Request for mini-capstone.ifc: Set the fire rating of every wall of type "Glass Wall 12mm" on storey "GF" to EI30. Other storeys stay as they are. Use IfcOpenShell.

First a look at what the model holds.

```python
import ifcopenshell
import ifcopenshell.util.element

model = ifcopenshell.open("mini-capstone.ifc")
print(model.schema)
storey = next(s for s in model.by_type("IfcBuildingStorey") if s.Name == "GF")
walls = [e for e in ifcopenshell.util.element.get_decomposition(storey) if e.is_a("IfcWall")]
seen = {}
for e in walls:
    element_type = ifcopenshell.util.element.get_type(e)
    key = (element_type.Name if element_type != e and element_type else None, ifcopenshell.util.element.get_pset(e, "Pset_WallCommon", "FireRating"))
    seen[key] = seen.get(key, 0) + 1
for (name, value), count in sorted(seen.items(), key=str):
    print(count, "x", name, "|", value)
```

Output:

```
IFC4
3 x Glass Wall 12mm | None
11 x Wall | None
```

```python
import ifcopenshell
import ifcopenshell.api.pset
import ifcopenshell.util.element

model = ifcopenshell.open("mini-capstone.ifc")

storey = next(s for s in model.by_type("IfcBuildingStorey") if s.Name == "GF")
walls = [e for e in ifcopenshell.util.element.get_decomposition(storey) if e.is_a("IfcWall")]

count = 0
for e in walls:
    element_type = ifcopenshell.util.element.get_type(e)
    if element_type in (None, e) or element_type.Name != "Glass Wall 12mm":
        continue
    # add_pset returns the element's existing set when there is one.
    pset = ifcopenshell.api.pset.add_pset(model, product=e, name="Pset_WallCommon")
    ifcopenshell.api.pset.edit_pset(model, pset=pset, properties={"FireRating": "EI30"})
    count += 1

print(count, "walls updated")

model.write("mini-capstone_v2.ifc")
```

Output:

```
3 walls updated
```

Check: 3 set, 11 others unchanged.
